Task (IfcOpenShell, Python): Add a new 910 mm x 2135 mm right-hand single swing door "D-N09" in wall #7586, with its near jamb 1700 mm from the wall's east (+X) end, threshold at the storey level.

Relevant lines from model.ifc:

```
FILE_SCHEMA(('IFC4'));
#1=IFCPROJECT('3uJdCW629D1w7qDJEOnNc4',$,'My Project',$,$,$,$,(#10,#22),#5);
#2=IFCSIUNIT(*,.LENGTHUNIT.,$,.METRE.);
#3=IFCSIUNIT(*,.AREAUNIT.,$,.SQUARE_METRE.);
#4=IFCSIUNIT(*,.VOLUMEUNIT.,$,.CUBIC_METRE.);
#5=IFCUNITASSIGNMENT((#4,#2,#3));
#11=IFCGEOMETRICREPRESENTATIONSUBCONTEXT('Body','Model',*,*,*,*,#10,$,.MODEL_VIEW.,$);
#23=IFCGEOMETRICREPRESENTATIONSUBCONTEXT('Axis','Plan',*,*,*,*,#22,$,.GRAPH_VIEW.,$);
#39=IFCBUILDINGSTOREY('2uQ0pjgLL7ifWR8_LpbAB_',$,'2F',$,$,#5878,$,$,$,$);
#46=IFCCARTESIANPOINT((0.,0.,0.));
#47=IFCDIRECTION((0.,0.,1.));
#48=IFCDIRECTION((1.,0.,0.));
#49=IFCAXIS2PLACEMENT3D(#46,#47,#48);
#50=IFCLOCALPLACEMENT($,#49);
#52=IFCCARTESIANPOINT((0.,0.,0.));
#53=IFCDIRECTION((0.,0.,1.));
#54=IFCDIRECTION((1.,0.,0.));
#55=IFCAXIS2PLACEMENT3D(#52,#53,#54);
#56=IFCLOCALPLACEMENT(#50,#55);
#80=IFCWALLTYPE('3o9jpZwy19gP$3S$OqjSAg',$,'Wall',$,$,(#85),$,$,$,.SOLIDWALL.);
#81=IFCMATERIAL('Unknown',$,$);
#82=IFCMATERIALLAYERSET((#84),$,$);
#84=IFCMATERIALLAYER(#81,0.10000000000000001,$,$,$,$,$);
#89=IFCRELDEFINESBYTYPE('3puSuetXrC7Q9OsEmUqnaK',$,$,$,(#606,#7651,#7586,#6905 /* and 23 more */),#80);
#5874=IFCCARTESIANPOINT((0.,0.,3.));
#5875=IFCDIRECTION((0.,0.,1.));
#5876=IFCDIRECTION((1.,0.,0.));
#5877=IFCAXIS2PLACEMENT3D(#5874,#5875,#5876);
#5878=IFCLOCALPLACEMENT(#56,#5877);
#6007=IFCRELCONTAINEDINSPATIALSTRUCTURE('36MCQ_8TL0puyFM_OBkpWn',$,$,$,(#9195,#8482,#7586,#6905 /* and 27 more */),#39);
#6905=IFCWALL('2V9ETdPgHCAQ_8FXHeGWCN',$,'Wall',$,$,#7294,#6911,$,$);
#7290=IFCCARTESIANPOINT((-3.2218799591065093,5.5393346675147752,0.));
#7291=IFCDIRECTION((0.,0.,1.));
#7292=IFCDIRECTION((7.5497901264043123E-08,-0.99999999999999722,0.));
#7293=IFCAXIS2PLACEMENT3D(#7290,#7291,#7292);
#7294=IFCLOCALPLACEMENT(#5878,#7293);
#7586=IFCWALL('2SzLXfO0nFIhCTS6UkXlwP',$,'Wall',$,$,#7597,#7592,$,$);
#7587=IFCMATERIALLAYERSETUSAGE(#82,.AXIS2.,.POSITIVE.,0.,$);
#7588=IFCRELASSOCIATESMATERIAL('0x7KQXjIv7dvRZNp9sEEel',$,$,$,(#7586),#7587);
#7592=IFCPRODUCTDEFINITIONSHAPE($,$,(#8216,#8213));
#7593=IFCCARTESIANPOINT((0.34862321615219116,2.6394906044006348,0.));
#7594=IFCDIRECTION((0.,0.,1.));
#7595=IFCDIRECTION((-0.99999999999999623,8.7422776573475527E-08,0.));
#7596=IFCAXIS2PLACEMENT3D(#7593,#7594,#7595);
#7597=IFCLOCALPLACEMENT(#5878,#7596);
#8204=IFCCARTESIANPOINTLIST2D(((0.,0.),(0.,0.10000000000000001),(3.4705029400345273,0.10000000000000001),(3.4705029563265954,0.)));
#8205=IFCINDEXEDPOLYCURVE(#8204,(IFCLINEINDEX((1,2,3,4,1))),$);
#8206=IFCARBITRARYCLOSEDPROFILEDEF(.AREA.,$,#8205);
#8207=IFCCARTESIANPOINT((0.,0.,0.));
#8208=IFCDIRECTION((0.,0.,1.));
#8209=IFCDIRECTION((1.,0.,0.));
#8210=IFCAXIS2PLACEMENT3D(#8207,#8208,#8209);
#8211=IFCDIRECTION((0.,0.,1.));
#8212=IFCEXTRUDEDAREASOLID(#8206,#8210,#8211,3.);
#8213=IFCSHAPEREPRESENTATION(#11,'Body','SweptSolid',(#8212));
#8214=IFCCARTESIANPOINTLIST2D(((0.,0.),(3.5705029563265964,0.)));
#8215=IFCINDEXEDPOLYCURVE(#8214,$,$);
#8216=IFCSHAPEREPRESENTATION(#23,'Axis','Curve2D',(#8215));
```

```python
import numpy as np
import ifcopenshell
import ifcopenshell.api.feature
import ifcopenshell.api.geometry
import ifcopenshell.api.root
import ifcopenshell.api.spatial
import ifcopenshell.geom
import ifcopenshell.util.element
import ifcopenshell.util.placement
import ifcopenshell.util.representation
import ifcopenshell.util.shape
import ifcopenshell.util.unit

model = ifcopenshell.open("model.ifc")
unit_scale = ifcopenshell.util.unit.calculate_unit_scale(model)
settings = ifcopenshell.geom.settings()


def volume(element):
    """Net volume in cubic metres, openings subtracted."""
    shape = ifcopenshell.geom.create_shape(settings, element)
    return ifcopenshell.util.shape.get_volume(shape.geometry)


wall = model.by_id(7586)
storey = ifcopenshell.util.element.get_container(wall, ifc_class="IfcBuildingStorey")
context = ifcopenshell.util.representation.get_context(model, "Model", "Body", "MODEL_VIEW")
before = volume(wall)

width, height, from_end, sill = 0.91, 2.135, 1.7, 0.0  # metres

# The wall runs along its own X axis, and the end named is its -X end.
wall_shape = ifcopenshell.geom.create_shape(settings, wall)
x, y, z = ifcopenshell.util.shape.get_vertices(wall_shape.geometry).T
start = x.min() + from_end
face, thickness = float(y.min()), float(y.max() - y.min())
wall_matrix = ifcopenshell.util.placement.get_local_placement(wall.ObjectPlacement)
level = ifcopenshell.util.placement.get_local_placement(storey.ObjectPlacement)[2, 3]


def in_wall(x, y):
    """Placement at x, y metres in the wall's axes, at sill height."""
    matrix = wall_matrix.copy()
    matrix[:, 3] = wall_matrix @ np.array([x / unit_scale, y / unit_scale, 0.0, 1.0])
    matrix[2, 3] = level + sill / unit_scale
    return matrix


# Opening: a box that overshoots both wall faces by 50 mm.
opening = ifcopenshell.api.root.create_entity(model, ifc_class="IfcOpeningElement", predefined_type="OPENING")
box = ifcopenshell.api.geometry.add_wall_representation(
    model, context=context, length=width, height=height, thickness=thickness + 0.1
)
ifcopenshell.api.geometry.assign_representation(model, product=opening, representation=box)
ifcopenshell.api.geometry.edit_object_placement(model, product=opening, matrix=in_wall(start, face - 0.05), is_si=False)
ifcopenshell.api.feature.add_feature(model, feature=opening, element=wall)

door = ifcopenshell.api.root.create_entity(model, ifc_class="IfcDoor", name="D-N09", predefined_type="DOOR")
door.OverallWidth, door.OverallHeight = width / unit_scale, height / unit_scale
door.OperationType = "SINGLE_SWING_RIGHT"
body = ifcopenshell.api.geometry.add_door_representation(
    model,
    context=context,
    overall_width=door.OverallWidth,
    overall_height=door.OverallHeight,
    operation_type="SINGLE_SWING_RIGHT",
    lining_properties={"LiningDepth": thickness / unit_scale, "ThresholdDepth": thickness / unit_scale},
)
ifcopenshell.api.geometry.assign_representation(model, product=door, representation=body)
ifcopenshell.api.spatial.assign_container(model, products=[door], relating_structure=storey)
ifcopenshell.api.feature.add_filling(model, opening=opening, element=door)

# The lining spans the wall, so the door starts at the wall face.
ifcopenshell.api.geometry.edit_object_placement(model, product=door, matrix=in_wall(start, face), is_si=False)

after = volume(wall)

print(f"wall volume {before:.3f} -> {after:.3f} m3")

model.write("model_rev.ifc")
```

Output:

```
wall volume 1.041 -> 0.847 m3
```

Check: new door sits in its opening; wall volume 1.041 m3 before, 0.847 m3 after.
